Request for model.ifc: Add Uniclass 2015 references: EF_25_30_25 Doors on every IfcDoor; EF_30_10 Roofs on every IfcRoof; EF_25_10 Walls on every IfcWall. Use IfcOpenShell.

First a look at what the model holds.

```python
import ifcopenshell

model = ifcopenshell.open("model.ifc")
print(model.schema)
print("classifications:", [c.Name for c in model.by_type("IfcClassification")])
for ifc_class in ("IfcDoor", "IfcRoof", "IfcStair", "IfcWall", "IfcWindow"):
    print(ifc_class, len(model.by_type(ifc_class)))
```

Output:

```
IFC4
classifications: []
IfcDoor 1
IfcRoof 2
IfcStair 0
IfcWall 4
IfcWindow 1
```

```python
import ifcopenshell
import ifcopenshell.api.classification

model = ifcopenshell.open("model.ifc")

system = ifcopenshell.api.classification.add_classification(model, classification="Uniclass 2015")

codes = {
    "IfcDoor": ("EF_25_30_25", "Doors"),
    "IfcRoof": ("EF_30_10", "Roofs"),
    "IfcWall": ("EF_25_10", "Walls"),
}
for ifc_class, (code, name) in codes.items():
    products = model.by_type(ifc_class)
    ifcopenshell.api.classification.add_reference(
        model, products=products, classification=system, identification=code, name=name
    )
    print(code, len(products))

model.write("model_edited.ifc")
```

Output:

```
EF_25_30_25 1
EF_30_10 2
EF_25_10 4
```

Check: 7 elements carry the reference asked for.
